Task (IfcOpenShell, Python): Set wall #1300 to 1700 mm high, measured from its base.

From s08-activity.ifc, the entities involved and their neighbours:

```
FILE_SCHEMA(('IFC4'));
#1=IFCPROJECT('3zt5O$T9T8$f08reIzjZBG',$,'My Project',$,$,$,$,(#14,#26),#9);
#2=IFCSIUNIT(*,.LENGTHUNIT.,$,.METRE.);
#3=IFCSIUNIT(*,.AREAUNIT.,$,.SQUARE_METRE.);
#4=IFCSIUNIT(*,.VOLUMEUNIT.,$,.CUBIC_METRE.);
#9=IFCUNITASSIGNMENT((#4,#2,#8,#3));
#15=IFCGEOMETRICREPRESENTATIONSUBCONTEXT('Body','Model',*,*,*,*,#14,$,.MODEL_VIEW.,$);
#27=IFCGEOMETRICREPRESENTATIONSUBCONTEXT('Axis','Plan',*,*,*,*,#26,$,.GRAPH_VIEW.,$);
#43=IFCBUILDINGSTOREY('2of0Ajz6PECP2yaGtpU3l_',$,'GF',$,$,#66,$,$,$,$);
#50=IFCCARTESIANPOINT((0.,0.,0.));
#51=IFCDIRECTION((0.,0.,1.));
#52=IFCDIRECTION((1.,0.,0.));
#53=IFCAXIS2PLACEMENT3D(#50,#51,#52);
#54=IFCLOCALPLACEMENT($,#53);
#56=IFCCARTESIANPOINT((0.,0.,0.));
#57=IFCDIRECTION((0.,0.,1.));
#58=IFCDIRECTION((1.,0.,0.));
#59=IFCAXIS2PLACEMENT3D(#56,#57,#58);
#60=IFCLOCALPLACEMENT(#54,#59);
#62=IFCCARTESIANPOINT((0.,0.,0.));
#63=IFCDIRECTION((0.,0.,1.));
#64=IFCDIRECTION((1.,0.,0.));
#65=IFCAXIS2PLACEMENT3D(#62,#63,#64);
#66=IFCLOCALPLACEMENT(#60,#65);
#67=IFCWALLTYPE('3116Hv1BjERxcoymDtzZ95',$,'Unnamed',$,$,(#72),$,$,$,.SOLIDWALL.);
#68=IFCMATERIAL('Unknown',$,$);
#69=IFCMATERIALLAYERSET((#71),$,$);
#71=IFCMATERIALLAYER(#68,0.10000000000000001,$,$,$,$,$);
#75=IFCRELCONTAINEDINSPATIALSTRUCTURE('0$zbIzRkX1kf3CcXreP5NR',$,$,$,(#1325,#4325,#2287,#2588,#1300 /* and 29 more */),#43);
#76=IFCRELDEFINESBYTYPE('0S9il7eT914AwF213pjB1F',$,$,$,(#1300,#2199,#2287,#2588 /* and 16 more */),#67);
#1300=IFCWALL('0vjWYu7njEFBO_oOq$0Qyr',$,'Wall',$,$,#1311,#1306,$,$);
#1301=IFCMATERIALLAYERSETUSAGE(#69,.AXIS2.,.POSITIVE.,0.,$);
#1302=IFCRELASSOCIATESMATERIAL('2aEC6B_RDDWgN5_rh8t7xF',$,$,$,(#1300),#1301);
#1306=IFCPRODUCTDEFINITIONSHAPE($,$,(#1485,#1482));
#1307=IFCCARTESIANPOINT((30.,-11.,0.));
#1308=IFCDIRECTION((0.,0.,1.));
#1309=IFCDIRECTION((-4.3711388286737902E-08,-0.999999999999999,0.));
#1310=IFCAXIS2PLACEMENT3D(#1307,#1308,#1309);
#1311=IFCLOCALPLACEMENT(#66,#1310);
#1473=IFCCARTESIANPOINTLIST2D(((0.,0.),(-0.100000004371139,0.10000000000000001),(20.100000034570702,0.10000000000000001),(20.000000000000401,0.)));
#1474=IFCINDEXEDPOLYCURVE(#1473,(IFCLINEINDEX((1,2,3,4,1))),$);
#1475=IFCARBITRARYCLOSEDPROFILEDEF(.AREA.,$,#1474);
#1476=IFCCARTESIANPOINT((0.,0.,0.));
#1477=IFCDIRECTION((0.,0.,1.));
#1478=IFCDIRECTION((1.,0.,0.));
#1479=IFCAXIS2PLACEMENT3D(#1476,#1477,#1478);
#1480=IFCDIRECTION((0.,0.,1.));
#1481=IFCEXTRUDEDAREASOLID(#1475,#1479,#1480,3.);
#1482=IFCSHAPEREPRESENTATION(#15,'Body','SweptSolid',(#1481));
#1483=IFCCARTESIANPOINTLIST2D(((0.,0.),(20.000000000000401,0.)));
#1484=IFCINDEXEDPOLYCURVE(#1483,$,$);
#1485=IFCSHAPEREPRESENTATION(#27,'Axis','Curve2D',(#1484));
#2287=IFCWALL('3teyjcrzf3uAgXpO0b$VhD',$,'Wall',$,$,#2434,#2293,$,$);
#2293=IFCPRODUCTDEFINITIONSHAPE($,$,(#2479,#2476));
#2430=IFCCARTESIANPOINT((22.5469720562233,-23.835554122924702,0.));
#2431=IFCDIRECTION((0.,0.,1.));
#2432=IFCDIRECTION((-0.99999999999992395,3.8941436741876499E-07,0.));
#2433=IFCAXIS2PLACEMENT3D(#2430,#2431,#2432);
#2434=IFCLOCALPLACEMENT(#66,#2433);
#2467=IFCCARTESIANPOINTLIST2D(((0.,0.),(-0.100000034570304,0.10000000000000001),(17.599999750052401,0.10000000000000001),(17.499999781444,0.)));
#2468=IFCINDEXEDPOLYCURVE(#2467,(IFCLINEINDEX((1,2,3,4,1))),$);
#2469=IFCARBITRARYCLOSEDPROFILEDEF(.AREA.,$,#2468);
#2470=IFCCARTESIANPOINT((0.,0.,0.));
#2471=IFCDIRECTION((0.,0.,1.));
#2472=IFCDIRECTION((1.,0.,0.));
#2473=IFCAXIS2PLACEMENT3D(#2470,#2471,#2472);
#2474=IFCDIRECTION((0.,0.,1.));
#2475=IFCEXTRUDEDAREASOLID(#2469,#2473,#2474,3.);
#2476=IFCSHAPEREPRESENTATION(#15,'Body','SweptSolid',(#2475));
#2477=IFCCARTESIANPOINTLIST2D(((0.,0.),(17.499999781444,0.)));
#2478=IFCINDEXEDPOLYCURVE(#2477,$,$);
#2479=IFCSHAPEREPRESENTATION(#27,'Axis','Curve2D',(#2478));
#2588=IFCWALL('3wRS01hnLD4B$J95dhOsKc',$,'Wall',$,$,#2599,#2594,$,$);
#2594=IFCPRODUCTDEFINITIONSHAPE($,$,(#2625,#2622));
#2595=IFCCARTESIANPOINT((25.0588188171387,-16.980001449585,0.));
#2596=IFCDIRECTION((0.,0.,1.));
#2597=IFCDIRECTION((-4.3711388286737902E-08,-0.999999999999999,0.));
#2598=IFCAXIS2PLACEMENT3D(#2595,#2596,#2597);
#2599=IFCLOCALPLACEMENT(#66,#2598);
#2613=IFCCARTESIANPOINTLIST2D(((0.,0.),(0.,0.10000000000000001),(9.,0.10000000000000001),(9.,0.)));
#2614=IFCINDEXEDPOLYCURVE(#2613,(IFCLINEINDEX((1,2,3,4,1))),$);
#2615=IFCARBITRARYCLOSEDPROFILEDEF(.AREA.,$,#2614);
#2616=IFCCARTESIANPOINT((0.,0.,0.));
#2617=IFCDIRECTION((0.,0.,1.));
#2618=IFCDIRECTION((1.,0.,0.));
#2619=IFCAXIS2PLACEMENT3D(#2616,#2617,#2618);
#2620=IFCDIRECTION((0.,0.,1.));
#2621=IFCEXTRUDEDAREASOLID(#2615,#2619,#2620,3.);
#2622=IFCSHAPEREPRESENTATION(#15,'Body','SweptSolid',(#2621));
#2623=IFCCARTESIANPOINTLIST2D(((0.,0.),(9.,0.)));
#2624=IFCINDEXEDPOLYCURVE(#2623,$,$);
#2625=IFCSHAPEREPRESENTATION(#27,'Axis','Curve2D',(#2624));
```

```python
import ifcopenshell
import ifcopenshell.geom
import ifcopenshell.util.representation
import ifcopenshell.util.shape
import ifcopenshell.util.unit

model = ifcopenshell.open("s08-activity.ifc")
unit_scale = ifcopenshell.util.unit.calculate_unit_scale(model)
settings = ifcopenshell.geom.settings()


def volume(element):
    """Net volume in cubic metres, openings subtracted."""
    shape = ifcopenshell.geom.create_shape(settings, element)
    return ifcopenshell.util.shape.get_volume(shape.geometry)


wall = model.by_guid("0vjWYu7njEFBO_oOq$0Qyr")
before = volume(wall)

body = ifcopenshell.util.representation.get_representation(wall, "Model", "Body")
solid = body.Items[0]
old_height = solid.Depth
solid.Depth = 1.7 / unit_scale
after = volume(wall)

print(f"height {old_height:g} -> {solid.Depth:g}, volume {before:.3f} -> {after:.3f} m3")

model.write("s08-activity_updated.ifc")
```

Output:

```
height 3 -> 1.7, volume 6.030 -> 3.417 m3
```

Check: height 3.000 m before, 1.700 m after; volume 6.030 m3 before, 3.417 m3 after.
